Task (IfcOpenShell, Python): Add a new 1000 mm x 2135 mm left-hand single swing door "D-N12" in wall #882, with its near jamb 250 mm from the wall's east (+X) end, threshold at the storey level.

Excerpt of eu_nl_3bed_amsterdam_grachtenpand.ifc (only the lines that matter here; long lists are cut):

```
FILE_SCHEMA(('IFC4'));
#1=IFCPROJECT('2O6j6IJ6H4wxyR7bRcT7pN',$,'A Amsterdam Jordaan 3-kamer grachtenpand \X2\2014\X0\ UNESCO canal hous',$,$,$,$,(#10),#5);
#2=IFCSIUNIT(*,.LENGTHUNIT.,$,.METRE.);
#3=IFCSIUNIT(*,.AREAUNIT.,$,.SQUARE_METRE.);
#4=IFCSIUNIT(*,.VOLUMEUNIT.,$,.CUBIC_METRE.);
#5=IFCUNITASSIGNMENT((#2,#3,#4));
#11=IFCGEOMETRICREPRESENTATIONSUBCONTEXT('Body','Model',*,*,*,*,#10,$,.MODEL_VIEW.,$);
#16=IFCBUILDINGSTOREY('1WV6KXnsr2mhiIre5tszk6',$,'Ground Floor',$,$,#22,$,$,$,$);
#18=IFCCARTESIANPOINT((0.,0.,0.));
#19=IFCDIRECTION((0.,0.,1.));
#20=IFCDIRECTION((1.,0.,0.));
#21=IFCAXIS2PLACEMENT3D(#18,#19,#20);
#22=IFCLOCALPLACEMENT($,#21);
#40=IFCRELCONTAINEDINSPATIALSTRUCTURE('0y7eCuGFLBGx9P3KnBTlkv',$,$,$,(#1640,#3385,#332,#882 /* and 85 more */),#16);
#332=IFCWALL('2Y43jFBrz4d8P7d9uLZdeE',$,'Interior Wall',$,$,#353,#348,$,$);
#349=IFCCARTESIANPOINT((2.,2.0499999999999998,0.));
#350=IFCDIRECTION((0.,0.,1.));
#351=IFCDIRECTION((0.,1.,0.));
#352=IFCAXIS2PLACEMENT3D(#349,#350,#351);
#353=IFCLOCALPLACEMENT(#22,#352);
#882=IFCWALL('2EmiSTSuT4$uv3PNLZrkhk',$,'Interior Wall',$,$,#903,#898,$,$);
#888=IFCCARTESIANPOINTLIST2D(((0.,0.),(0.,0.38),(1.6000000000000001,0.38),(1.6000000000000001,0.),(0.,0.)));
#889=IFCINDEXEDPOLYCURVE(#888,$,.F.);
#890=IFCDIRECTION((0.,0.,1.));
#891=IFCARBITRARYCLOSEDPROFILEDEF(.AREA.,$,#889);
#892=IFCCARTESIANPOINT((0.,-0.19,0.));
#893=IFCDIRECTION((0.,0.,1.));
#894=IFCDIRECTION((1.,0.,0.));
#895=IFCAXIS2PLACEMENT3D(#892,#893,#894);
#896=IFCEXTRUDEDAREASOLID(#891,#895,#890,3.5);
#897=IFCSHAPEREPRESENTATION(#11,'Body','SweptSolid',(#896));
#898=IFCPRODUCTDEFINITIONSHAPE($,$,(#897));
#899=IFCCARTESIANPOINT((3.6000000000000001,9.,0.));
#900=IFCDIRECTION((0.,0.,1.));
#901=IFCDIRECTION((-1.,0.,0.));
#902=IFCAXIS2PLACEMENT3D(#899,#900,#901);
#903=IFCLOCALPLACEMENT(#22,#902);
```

```python
import numpy as np
import ifcopenshell
import ifcopenshell.api.feature
import ifcopenshell.api.geometry
import ifcopenshell.api.root
import ifcopenshell.api.spatial
import ifcopenshell.geom
import ifcopenshell.util.element
import ifcopenshell.util.placement
import ifcopenshell.util.representation
import ifcopenshell.util.shape
import ifcopenshell.util.unit

model = ifcopenshell.open("eu_nl_3bed_amsterdam_grachtenpand.ifc")
unit_scale = ifcopenshell.util.unit.calculate_unit_scale(model)
settings = ifcopenshell.geom.settings()


def volume(element):
    """Net volume in cubic metres, openings subtracted."""
    shape = ifcopenshell.geom.create_shape(settings, element)
    return ifcopenshell.util.shape.get_volume(shape.geometry)


wall = model.by_guid("2EmiSTSuT4$uv3PNLZrkhk")
storey = ifcopenshell.util.element.get_container(wall, ifc_class="IfcBuildingStorey")
context = ifcopenshell.util.representation.get_context(model, "Model", "Body", "MODEL_VIEW")
before = volume(wall)

width, height, from_end, sill = 1, 2.135, 0.25, 0.0  # metres

# The wall runs along its own X axis, and the end named is its -X end.
wall_shape = ifcopenshell.geom.create_shape(settings, wall)
x, y, z = ifcopenshell.util.shape.get_vertices(wall_shape.geometry).T
start = x.min() + from_end
face, thickness = float(y.min()), float(y.max() - y.min())
wall_matrix = ifcopenshell.util.placement.get_local_placement(wall.ObjectPlacement)
level = ifcopenshell.util.placement.get_local_placement(storey.ObjectPlacement)[2, 3]


def in_wall(x, y):
    """Placement at x, y metres in the wall's axes, at sill height."""
    matrix = wall_matrix.copy()
    matrix[:, 3] = wall_matrix @ np.array([x / unit_scale, y / unit_scale, 0.0, 1.0])
    matrix[2, 3] = level + sill / unit_scale
    return matrix


# Opening: a box that overshoots both wall faces by 50 mm.
opening = ifcopenshell.api.root.create_entity(model, ifc_class="IfcOpeningElement", predefined_type="OPENING")
box = ifcopenshell.api.geometry.add_wall_representation(
    model, context=context, length=width, height=height, thickness=thickness + 0.1
)
ifcopenshell.api.geometry.assign_representation(model, product=opening, representation=box)
ifcopenshell.api.geometry.edit_object_placement(model, product=opening, matrix=in_wall(start, face - 0.05), is_si=False)
ifcopenshell.api.feature.add_feature(model, feature=opening, element=wall)

door = ifcopenshell.api.root.create_entity(model, ifc_class="IfcDoor", name="D-N12", predefined_type="DOOR")
door.OverallWidth, door.OverallHeight = width / unit_scale, height / unit_scale
door.OperationType = "SINGLE_SWING_LEFT"
body = ifcopenshell.api.geometry.add_door_representation(
    model,
    context=context,
    overall_width=door.OverallWidth,
    overall_height=door.OverallHeight,
    operation_type="SINGLE_SWING_LEFT",
    lining_properties={"LiningDepth": thickness / unit_scale, "ThresholdDepth": thickness / unit_scale},
)
ifcopenshell.api.geometry.assign_representation(model, product=door, representation=body)
ifcopenshell.api.spatial.assign_container(model, products=[door], relating_structure=storey)
ifcopenshell.api.feature.add_filling(model, opening=opening, element=door)

# The lining spans the wall, so the door starts at the wall face.
ifcopenshell.api.geometry.edit_object_placement(model, product=door, matrix=in_wall(start, face), is_si=False)

after = volume(wall)

print(f"wall volume {before:.3f} -> {after:.3f} m3")

model.write("eu_nl_3bed_amsterdam_grachtenpand_edited.ifc")
```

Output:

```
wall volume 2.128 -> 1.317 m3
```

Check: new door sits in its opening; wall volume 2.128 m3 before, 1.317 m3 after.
